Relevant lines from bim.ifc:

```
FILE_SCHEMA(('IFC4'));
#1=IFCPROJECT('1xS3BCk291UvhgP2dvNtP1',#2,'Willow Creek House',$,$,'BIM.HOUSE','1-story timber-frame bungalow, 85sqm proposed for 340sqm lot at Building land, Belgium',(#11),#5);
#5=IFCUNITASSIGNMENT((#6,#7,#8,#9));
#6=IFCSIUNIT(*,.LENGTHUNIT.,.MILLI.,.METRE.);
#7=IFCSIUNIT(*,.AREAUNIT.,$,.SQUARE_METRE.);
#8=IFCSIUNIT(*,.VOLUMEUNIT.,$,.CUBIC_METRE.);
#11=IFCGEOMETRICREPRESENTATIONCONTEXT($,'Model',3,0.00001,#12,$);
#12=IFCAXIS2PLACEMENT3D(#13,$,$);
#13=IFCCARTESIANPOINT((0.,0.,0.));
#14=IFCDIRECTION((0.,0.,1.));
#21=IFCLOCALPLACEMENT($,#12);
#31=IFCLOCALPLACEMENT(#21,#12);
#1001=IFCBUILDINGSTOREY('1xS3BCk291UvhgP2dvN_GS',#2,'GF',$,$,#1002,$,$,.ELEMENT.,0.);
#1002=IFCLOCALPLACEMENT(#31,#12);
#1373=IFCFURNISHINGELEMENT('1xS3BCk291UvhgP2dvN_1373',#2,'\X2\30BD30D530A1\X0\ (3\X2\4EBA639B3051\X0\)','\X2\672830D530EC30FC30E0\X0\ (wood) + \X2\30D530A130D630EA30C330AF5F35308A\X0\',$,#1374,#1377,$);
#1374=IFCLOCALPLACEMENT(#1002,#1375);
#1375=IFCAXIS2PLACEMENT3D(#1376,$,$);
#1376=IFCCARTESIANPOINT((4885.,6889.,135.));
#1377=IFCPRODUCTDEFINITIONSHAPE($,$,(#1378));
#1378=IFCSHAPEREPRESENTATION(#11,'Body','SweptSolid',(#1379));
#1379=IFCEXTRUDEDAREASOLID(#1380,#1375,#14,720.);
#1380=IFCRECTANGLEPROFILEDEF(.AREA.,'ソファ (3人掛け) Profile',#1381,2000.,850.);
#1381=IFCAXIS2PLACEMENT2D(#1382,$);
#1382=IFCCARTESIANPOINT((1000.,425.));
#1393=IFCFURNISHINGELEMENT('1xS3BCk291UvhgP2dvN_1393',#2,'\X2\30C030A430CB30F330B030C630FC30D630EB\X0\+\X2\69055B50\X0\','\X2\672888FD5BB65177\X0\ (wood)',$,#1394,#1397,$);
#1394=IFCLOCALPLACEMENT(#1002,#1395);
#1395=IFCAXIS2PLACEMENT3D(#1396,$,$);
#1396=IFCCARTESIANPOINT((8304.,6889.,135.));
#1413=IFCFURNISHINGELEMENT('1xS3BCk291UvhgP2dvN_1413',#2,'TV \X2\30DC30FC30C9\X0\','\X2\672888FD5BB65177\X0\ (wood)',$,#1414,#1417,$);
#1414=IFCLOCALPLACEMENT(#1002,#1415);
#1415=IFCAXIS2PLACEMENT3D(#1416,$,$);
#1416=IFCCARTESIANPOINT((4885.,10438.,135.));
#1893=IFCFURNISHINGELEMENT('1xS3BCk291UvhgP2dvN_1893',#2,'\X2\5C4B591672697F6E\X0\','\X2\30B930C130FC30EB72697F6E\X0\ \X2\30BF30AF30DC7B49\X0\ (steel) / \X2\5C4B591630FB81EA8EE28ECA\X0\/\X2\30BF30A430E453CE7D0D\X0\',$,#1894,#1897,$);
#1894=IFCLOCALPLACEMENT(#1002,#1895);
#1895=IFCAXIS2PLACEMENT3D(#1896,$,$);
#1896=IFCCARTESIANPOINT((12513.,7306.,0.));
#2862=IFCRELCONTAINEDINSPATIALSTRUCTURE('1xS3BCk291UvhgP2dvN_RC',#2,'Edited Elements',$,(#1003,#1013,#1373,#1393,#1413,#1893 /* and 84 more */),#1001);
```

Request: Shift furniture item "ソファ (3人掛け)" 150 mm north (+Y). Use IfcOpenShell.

```python
import ifcopenshell
import ifcopenshell.api.geometry
import ifcopenshell.util.placement

model = ifcopenshell.open("bim.ifc")

item = model.by_guid("1xS3BCk291UvhgP2dvN_1373")
matrix = ifcopenshell.util.placement.get_local_placement(item.ObjectPlacement)
matrix[1, 3] += 150.0
ifcopenshell.api.geometry.edit_object_placement(model, product=item, matrix=matrix, is_si=False)

print(ifcopenshell.util.placement.get_local_placement(item.ObjectPlacement).round(3) + 0.0)

model.write("bim_updated.ifc")
```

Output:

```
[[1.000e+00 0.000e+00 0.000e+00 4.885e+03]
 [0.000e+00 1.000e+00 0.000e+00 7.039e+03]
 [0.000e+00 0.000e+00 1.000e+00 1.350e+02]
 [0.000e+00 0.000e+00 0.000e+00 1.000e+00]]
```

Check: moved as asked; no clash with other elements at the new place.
